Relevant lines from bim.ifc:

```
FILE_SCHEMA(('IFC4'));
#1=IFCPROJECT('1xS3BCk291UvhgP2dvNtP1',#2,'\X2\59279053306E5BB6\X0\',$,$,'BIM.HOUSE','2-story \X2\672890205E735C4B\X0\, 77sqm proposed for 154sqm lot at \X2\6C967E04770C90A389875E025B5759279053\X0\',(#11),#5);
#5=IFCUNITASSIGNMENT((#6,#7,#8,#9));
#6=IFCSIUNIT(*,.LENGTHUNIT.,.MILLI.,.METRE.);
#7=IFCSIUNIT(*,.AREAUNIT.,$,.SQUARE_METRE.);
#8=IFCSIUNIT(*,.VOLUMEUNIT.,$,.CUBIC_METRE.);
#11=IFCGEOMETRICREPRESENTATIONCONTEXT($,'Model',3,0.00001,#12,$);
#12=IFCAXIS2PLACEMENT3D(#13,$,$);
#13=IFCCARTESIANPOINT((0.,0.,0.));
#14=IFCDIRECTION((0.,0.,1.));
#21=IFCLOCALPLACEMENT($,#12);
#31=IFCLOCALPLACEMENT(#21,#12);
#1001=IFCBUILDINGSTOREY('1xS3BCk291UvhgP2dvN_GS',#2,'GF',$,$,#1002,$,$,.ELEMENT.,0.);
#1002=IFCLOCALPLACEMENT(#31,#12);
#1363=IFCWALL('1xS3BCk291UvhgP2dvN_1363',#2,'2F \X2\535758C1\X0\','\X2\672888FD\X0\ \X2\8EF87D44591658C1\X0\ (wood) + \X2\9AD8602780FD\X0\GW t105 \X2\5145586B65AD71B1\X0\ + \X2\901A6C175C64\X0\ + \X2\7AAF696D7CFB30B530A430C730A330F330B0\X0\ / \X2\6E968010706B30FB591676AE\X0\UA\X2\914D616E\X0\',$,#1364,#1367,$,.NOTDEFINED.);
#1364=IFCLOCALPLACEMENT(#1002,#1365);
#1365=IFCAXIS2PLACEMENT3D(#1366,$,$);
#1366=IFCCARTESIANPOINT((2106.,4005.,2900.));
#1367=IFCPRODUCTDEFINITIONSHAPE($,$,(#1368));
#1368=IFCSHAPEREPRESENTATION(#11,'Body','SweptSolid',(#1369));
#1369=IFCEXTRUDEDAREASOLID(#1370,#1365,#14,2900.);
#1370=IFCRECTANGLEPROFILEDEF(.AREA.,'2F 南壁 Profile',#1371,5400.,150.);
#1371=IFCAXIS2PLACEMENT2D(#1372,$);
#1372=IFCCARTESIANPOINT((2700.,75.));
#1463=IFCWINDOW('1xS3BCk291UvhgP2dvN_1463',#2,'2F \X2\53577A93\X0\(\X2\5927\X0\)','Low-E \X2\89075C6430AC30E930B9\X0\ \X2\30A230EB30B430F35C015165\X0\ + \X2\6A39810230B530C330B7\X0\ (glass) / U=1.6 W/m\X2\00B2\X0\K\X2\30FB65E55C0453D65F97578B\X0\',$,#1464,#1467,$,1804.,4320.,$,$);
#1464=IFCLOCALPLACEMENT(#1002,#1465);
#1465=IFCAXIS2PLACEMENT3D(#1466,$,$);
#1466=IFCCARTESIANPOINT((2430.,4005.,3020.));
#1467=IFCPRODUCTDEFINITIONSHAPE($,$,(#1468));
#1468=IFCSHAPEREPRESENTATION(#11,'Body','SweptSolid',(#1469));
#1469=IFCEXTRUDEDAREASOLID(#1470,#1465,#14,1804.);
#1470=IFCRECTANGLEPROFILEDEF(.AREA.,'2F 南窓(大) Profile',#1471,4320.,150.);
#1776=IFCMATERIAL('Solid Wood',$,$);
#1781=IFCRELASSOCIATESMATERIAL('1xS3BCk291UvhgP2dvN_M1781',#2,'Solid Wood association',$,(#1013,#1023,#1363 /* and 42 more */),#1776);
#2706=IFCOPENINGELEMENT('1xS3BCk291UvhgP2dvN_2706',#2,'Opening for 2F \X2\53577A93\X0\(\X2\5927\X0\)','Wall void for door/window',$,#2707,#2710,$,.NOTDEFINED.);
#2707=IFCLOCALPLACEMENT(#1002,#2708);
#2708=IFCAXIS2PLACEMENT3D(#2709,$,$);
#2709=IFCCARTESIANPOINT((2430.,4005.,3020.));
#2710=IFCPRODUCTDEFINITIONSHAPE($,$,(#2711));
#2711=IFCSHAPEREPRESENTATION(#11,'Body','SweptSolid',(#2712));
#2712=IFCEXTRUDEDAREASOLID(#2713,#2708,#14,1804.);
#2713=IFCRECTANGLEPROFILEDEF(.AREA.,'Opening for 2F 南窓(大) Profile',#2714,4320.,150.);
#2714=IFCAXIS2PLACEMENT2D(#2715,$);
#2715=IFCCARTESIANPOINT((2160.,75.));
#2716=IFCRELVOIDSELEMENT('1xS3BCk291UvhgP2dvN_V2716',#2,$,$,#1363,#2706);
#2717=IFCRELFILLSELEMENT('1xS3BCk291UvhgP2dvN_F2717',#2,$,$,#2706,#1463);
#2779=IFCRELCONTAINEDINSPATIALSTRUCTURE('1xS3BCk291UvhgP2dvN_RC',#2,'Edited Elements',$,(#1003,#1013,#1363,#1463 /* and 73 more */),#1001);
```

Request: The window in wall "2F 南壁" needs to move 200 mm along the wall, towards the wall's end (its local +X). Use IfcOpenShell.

```python
import ifcopenshell
import ifcopenshell.api.geometry
import ifcopenshell.util.placement

model = ifcopenshell.open("bim.ifc")

window = model.by_guid("1xS3BCk291UvhgP2dvN_1463")
opening = window.FillsVoids[0].RelatingOpeningElement
wall = opening.VoidsElements[0].RelatingBuildingElement

wall_matrix = ifcopenshell.util.placement.get_local_placement(wall.ObjectPlacement)
shift = wall_matrix[:3, 0] * 200.0
before = ifcopenshell.util.placement.get_local_placement(window.ObjectPlacement)[:3, 3].copy()

# The window is not placed relative to its opening, so move both.
for product in (opening, window):
    matrix = ifcopenshell.util.placement.get_local_placement(product.ObjectPlacement)
    matrix[:3, 3] += shift
    ifcopenshell.api.geometry.edit_object_placement(model, product=product, matrix=matrix, is_si=False)

after = ifcopenshell.util.placement.get_local_placement(window.ObjectPlacement)[:3, 3]
print("window moved by", (after - before).round(3) + 0.0)

model.write("bim_v2.ifc")
```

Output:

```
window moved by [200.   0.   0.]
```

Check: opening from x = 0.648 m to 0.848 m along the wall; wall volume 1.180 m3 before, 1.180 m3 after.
